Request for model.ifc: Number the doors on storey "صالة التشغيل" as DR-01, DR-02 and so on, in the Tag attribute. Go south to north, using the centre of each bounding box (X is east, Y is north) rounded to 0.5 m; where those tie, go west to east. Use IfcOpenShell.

First a look at what the model holds.

```python
import ifcopenshell
import ifcopenshell.util.element
import ifcopenshell.util.placement

model = ifcopenshell.open("model.ifc")
print(model.schema)
storey = next(s for s in model.by_type("IfcBuildingStorey") if s.Name == "صالة التشغيل")
doors = [e for e in ifcopenshell.util.element.get_decomposition(storey) if e.is_a("IfcDoor")]
for e in sorted(doors, key=lambda e: e.id()):
    origin = ifcopenshell.util.placement.get_local_placement(e.ObjectPlacement)[:3, 3]
    print(e.id(), e.Tag, e.Name, origin.round(2) + 0.0, sep=" | ")
```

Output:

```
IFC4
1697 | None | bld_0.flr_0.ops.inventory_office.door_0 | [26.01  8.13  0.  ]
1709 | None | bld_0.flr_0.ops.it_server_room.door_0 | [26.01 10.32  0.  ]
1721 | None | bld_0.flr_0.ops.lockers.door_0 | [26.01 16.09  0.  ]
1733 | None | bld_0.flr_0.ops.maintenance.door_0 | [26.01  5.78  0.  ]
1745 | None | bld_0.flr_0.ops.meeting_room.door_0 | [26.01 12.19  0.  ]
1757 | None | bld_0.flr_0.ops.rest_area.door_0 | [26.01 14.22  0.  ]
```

```python
import ifcopenshell
import ifcopenshell.geom
import ifcopenshell.util.element
import ifcopenshell.util.shape

model = ifcopenshell.open("model.ifc")
settings = ifcopenshell.geom.settings()
settings.set("use-world-coords", True)


def centre(element):
    shape = ifcopenshell.geom.create_shape(settings, element)
    return ifcopenshell.util.shape.get_bbox_centroid(shape.geometry)


storey = next(s for s in model.by_type("IfcBuildingStorey") if s.Name == "صالة التشغيل")
doors = [e for e in ifcopenshell.util.element.get_decomposition(storey) if e.is_a("IfcDoor")]

# Insertion points can sit at a corner or the storey origin, so sort by the geometry (in metres).
centres = {e: centre(e) for e in doors}
doors.sort(key=lambda e: (round(centres[e][1] / 0.5), centres[e][0]))

for i, e in enumerate(doors, start=1):
    number = f"DR-{i:02d}"
    e.Tag = number
    print(e.id(), number)

model.write("model-out.ifc")
```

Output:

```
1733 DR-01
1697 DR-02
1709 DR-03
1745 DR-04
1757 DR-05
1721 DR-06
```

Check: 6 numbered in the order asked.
